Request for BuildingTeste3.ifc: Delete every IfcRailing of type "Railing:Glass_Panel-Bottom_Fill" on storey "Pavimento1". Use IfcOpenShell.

First a look at what the model holds.

```python
import ifcopenshell
import ifcopenshell.util.element

model = ifcopenshell.open("BuildingTeste3.ifc")
print(model.schema)
storey = next(s for s in model.by_type("IfcBuildingStorey") if s.Name == "Pavimento1")
railings = [e for e in ifcopenshell.util.element.get_decomposition(storey) if e.is_a("IfcRailing")]
seen = {}
for e in railings:
    element_type = ifcopenshell.util.element.get_type(e)
    name = element_type.Name if element_type not in (None, e) else None
    seen[name] = seen.get(name, 0) + 1
for name, count in sorted(seen.items(), key=str):
    print(count, "x", name)
```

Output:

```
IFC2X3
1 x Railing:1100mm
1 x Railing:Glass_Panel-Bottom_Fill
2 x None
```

```python
import ifcopenshell
import ifcopenshell.api.root
import ifcopenshell.util.element

model = ifcopenshell.open("BuildingTeste3.ifc")

storey = next(s for s in model.by_type("IfcBuildingStorey") if s.Name == "Pavimento1")
railings = [e for e in ifcopenshell.util.element.get_decomposition(storey) if e.is_a("IfcRailing")]
targets = [e for e in railings if (t := ifcopenshell.util.element.get_type(e)) not in (None, e) and t.Name == "Railing:Glass_Panel-Bottom_Fill"]

for e in targets:
    ifcopenshell.api.root.remove_product(model, product=e)
print(len(targets), "removed")

model.write("BuildingTeste3_rev.ifc")
```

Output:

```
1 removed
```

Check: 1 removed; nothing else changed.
